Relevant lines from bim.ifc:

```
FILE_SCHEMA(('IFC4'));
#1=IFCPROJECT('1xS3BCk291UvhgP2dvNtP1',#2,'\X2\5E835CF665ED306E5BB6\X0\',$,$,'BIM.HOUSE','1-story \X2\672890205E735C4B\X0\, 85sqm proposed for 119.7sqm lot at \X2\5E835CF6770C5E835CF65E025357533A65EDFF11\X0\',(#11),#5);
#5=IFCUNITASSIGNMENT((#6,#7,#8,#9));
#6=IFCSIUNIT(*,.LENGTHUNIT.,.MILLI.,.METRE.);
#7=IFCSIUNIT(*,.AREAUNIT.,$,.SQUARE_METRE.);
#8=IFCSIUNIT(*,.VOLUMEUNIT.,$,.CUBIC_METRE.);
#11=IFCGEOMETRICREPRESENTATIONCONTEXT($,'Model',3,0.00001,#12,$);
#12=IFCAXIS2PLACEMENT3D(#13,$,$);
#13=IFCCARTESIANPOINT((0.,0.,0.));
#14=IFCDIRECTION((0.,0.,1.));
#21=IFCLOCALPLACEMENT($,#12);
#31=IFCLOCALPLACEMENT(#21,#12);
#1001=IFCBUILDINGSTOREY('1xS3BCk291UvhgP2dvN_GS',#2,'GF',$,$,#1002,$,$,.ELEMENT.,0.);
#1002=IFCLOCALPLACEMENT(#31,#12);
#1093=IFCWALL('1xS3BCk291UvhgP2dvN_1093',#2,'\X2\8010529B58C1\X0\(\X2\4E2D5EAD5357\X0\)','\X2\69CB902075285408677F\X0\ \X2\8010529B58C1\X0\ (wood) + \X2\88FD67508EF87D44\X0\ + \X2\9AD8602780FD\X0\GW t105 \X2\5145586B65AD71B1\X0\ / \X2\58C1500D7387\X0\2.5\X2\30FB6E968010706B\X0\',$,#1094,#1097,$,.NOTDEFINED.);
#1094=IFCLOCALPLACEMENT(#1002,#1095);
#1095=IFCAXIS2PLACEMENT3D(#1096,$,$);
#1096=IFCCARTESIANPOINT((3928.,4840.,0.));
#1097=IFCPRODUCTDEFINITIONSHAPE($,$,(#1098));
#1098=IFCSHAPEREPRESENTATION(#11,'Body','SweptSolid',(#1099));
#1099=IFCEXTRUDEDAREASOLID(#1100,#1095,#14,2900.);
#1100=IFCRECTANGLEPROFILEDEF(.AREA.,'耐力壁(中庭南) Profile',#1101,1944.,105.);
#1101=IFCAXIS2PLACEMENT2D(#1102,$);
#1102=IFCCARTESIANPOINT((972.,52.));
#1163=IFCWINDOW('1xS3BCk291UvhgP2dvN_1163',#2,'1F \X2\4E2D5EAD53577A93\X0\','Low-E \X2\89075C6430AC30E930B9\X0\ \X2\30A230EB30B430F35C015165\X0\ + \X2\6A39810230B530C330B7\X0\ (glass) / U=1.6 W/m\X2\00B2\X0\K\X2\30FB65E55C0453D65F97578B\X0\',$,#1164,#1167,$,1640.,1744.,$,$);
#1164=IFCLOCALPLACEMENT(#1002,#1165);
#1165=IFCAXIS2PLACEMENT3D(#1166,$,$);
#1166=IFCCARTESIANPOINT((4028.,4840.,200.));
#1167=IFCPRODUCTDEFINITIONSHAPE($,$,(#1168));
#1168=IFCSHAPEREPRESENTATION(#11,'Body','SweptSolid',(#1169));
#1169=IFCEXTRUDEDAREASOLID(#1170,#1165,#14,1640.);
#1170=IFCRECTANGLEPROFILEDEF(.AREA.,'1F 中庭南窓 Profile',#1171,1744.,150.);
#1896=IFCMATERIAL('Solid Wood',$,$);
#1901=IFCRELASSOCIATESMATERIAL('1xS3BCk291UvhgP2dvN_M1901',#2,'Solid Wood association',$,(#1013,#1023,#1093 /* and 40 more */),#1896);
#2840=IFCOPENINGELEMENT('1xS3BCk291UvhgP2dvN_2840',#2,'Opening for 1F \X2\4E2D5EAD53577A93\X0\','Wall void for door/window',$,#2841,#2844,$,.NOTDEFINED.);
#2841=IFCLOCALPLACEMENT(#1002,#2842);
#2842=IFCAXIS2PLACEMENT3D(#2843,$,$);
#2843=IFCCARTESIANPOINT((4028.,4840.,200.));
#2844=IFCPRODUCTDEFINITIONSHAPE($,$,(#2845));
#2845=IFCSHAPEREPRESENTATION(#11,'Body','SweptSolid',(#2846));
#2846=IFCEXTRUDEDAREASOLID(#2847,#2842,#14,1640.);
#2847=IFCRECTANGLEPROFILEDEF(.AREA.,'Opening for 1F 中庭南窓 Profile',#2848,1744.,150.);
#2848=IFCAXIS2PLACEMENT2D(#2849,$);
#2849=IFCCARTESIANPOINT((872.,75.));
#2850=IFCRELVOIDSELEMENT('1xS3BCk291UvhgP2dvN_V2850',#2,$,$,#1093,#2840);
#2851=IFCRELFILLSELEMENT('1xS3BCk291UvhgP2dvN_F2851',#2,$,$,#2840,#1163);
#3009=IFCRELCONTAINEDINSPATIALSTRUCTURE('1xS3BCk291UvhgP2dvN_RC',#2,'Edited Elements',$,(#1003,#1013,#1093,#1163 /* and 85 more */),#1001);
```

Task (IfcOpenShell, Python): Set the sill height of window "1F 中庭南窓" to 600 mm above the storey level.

```python
import numpy as np
import ifcopenshell
import ifcopenshell.api.geometry
import ifcopenshell.geom
import ifcopenshell.util.element
import ifcopenshell.util.placement
import ifcopenshell.util.shape
import ifcopenshell.util.unit

model = ifcopenshell.open("bim.ifc")
unit_scale = ifcopenshell.util.unit.calculate_unit_scale(model)

window = model.by_guid("1xS3BCk291UvhgP2dvN_1163")
opening = window.FillsVoids[0].RelatingOpeningElement
storey = ifcopenshell.util.element.get_container(window, ifc_class="IfcBuildingStorey")
level = ifcopenshell.util.placement.get_local_placement(storey.ObjectPlacement)[2, 3]

# The opening's origin need not be at the sill, so measure its lowest point.
shape = ifcopenshell.geom.create_shape(ifcopenshell.geom.settings(), opening)
bottom = ifcopenshell.util.shape.get_shape_bottom_elevation(shape, shape.geometry) / unit_scale
dz = level + 0.6 / unit_scale - bottom

shift = np.array([0.0, 0.0, dz])
# The window is not placed relative to its opening, so move both.
for product in (opening, window):
    matrix = ifcopenshell.util.placement.get_local_placement(product.ObjectPlacement)
    matrix[:3, 3] += shift
    ifcopenshell.api.geometry.edit_object_placement(model, product=product, matrix=matrix, is_si=False)

print(f"moved by {dz * unit_scale:+.3f} m")

model.write("bim-out.ifc")
```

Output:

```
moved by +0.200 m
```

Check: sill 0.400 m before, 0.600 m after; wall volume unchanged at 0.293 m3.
